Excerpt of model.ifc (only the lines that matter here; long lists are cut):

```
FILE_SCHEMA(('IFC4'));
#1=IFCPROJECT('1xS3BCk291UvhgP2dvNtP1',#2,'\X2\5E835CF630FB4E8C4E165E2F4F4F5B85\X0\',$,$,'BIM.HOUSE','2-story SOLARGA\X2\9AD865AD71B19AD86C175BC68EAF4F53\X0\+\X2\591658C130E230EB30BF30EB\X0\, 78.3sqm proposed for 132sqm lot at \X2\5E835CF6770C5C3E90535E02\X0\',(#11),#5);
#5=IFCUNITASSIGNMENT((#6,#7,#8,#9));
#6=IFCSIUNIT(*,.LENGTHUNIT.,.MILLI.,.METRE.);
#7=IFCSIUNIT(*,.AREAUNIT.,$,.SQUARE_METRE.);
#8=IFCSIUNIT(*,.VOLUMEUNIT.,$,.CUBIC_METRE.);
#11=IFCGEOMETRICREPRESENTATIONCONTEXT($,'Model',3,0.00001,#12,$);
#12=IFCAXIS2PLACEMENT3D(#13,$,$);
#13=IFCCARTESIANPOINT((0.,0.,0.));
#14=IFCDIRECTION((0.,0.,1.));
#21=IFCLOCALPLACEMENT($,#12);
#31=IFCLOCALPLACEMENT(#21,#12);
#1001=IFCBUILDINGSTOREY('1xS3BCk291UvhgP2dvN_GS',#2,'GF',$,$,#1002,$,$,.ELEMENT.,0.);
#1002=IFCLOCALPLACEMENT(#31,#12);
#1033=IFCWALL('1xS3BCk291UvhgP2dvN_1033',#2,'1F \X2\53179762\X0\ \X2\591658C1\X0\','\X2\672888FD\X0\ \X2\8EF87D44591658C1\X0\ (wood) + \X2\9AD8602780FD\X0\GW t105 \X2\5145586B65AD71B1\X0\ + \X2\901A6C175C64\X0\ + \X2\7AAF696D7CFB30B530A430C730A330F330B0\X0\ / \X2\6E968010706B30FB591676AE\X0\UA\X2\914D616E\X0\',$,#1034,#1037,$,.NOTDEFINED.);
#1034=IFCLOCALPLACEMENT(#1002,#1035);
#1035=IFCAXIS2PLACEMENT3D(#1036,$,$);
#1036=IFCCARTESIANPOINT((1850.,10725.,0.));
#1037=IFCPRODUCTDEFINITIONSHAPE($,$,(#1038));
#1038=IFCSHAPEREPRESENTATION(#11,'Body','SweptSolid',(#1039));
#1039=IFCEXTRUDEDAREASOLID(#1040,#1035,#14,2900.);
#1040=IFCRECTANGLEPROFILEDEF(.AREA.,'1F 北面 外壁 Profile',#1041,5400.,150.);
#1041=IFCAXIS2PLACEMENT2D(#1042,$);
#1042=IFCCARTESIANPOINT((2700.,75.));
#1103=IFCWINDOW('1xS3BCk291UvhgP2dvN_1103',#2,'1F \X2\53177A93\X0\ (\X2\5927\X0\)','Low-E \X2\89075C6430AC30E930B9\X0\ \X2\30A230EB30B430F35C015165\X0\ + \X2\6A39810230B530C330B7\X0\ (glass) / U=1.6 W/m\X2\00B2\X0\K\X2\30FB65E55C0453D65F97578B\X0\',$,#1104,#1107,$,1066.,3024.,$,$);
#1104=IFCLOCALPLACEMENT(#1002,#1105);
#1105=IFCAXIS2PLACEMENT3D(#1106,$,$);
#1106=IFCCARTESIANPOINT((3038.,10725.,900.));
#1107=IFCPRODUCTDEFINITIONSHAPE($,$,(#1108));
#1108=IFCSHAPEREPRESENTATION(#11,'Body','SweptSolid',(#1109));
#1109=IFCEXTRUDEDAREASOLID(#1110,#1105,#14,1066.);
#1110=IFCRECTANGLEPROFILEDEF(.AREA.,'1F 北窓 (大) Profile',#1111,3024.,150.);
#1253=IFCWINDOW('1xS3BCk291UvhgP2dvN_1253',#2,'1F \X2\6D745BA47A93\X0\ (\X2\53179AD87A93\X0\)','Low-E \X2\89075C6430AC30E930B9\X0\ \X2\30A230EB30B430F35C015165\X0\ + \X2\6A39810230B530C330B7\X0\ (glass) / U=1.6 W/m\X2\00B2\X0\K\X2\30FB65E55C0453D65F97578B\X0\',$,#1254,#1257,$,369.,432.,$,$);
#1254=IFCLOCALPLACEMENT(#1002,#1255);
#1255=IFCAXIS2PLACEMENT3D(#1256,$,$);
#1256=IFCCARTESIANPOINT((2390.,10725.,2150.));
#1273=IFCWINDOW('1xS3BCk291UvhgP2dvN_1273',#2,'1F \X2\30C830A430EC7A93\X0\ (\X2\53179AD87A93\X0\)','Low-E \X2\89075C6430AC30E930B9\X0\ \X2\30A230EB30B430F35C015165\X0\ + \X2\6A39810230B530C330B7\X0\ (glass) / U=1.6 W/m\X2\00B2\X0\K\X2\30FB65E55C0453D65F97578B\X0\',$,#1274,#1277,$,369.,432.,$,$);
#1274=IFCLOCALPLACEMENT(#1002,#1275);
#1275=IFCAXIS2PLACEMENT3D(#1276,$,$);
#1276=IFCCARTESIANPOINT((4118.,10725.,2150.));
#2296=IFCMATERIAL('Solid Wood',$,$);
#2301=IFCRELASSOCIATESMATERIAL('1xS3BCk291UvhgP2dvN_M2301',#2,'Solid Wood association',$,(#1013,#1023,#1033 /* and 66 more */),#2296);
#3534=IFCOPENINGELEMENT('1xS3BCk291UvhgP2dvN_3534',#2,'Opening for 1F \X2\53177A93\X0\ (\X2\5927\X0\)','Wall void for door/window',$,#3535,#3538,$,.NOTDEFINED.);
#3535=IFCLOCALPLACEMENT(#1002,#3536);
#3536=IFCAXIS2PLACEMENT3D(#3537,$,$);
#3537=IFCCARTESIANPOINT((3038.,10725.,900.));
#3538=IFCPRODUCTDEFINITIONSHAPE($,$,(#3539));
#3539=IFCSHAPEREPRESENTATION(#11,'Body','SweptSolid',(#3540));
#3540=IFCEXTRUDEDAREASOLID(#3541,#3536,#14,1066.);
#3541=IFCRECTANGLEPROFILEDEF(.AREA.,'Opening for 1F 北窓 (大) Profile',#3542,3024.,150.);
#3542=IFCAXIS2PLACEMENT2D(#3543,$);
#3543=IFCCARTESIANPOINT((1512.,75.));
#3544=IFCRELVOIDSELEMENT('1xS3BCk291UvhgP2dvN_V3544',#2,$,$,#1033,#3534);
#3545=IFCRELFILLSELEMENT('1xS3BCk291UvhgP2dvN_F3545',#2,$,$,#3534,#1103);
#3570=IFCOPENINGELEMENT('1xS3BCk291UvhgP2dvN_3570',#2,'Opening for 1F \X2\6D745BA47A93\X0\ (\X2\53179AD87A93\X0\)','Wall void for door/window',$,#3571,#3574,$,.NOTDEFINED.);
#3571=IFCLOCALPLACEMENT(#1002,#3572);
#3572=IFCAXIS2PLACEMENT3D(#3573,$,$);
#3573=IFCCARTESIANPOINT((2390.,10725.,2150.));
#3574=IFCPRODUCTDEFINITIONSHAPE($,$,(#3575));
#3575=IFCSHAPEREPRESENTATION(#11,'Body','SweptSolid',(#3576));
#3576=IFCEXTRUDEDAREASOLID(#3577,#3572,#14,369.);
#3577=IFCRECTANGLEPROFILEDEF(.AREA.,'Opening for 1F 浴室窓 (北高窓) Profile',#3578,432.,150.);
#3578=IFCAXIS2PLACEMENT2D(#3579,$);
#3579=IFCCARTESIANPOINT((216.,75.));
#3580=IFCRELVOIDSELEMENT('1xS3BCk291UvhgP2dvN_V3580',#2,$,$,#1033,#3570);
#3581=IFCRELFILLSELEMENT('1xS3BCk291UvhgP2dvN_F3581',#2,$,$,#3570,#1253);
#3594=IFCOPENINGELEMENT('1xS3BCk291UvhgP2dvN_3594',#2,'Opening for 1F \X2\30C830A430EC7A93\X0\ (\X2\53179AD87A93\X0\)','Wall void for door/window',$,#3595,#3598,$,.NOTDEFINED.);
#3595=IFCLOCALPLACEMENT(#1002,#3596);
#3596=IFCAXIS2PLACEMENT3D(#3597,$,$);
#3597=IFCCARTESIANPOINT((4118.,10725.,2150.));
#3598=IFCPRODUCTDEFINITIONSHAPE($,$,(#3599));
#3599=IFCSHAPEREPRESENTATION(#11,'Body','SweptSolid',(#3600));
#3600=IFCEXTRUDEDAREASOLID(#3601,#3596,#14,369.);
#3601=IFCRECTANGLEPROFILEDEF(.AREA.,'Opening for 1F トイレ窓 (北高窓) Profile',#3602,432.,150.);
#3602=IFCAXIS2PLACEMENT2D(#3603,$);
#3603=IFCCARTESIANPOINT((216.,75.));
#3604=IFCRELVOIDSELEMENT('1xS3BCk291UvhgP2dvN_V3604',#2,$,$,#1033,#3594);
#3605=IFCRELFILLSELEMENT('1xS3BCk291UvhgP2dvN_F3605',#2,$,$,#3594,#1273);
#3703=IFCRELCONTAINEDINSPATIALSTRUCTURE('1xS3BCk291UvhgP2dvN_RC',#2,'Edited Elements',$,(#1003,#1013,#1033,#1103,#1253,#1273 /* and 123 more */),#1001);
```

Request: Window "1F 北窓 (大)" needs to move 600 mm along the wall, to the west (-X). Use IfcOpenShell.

```python
import ifcopenshell
import ifcopenshell.api.geometry
import ifcopenshell.util.placement

model = ifcopenshell.open("model.ifc")

window = model.by_guid("1xS3BCk291UvhgP2dvN_1103")
opening = window.FillsVoids[0].RelatingOpeningElement
wall = opening.VoidsElements[0].RelatingBuildingElement

wall_matrix = ifcopenshell.util.placement.get_local_placement(wall.ObjectPlacement)
shift = wall_matrix[:3, 0] * -600.0
before = ifcopenshell.util.placement.get_local_placement(window.ObjectPlacement)[:3, 3].copy()

# The window is not placed relative to its opening, so move both.
for product in (opening, window):
    matrix = ifcopenshell.util.placement.get_local_placement(product.ObjectPlacement)
    matrix[:3, 3] += shift
    ifcopenshell.api.geometry.edit_object_placement(model, product=product, matrix=matrix, is_si=False)

after = ifcopenshell.util.placement.get_local_placement(window.ObjectPlacement)[:3, 3]
print("window moved by", (after - before).round(3) + 0.0)

model.write("model_v2.ifc")
```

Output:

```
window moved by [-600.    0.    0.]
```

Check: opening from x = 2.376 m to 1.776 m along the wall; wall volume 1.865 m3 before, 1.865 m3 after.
